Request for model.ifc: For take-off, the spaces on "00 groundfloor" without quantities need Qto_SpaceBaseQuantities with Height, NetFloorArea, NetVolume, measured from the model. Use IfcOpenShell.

First a look at what the model holds.

```python
import ifcopenshell
import ifcopenshell.util.element
import ifcopenshell.util.unit

model = ifcopenshell.open("model.ifc")
print(model.schema)
for unit_type in ("LENGTHUNIT", "AREAUNIT", "VOLUMEUNIT"):
    print(unit_type, ifcopenshell.util.unit.calculate_unit_scale(model, unit_type))
storey = next(s for s in model.by_type("IfcBuildingStorey") if s.Name == "00 groundfloor")
spaces = [e for e in ifcopenshell.util.element.get_decomposition(storey) if e.is_a("IfcSpace")]
for e in sorted(spaces, key=lambda e: e.id()):
    print(e.id(), e.is_a(), e.Name, list(ifcopenshell.util.element.get_psets(e, qtos_only=True)), sep=" | ")
```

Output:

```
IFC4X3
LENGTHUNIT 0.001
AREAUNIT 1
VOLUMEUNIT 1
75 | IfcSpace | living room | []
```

```python
import ifcopenshell
import ifcopenshell.api.pset
import ifcopenshell.geom
import ifcopenshell.util.element
import ifcopenshell.util.shape
import ifcopenshell.util.unit

model = ifcopenshell.open("model.ifc")
unit_scale = ifcopenshell.util.unit.calculate_unit_scale(model)
area_scale = ifcopenshell.util.unit.calculate_unit_scale(model, "AREAUNIT")
volume_scale = ifcopenshell.util.unit.calculate_unit_scale(model, "VOLUMEUNIT")
settings = ifcopenshell.geom.settings()

storey = next(s for s in model.by_type("IfcBuildingStorey") if s.Name == "00 groundfloor")
spaces = [e for e in ifcopenshell.util.element.get_decomposition(storey) if e.is_a("IfcSpace")]

for e in sorted(spaces, key=lambda e: e.id()):
    if ifcopenshell.util.element.get_psets(e, qtos_only=True, should_inherit=False):
        continue
    # Geometry comes back in metres, in the element's own axes.
    shape = ifcopenshell.geom.create_shape(settings, e)
    values = {
        "Height": ifcopenshell.util.shape.get_z(shape.geometry) / unit_scale,
        "NetFloorArea": ifcopenshell.util.shape.get_footprint_area(shape.geometry) / area_scale,
        "NetVolume": ifcopenshell.util.shape.get_volume(shape.geometry) / volume_scale,
    }
    qto = ifcopenshell.api.pset.add_qto(model, product=e, name="Qto_SpaceBaseQuantities")
    ifcopenshell.api.pset.edit_qto(model, qto=qto, properties=values)
    print(e.id(), {k: round(v, 3) for k, v in values.items()})

model.write("model_rev.ifc")
```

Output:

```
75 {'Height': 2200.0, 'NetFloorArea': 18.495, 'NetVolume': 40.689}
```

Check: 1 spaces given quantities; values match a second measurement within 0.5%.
